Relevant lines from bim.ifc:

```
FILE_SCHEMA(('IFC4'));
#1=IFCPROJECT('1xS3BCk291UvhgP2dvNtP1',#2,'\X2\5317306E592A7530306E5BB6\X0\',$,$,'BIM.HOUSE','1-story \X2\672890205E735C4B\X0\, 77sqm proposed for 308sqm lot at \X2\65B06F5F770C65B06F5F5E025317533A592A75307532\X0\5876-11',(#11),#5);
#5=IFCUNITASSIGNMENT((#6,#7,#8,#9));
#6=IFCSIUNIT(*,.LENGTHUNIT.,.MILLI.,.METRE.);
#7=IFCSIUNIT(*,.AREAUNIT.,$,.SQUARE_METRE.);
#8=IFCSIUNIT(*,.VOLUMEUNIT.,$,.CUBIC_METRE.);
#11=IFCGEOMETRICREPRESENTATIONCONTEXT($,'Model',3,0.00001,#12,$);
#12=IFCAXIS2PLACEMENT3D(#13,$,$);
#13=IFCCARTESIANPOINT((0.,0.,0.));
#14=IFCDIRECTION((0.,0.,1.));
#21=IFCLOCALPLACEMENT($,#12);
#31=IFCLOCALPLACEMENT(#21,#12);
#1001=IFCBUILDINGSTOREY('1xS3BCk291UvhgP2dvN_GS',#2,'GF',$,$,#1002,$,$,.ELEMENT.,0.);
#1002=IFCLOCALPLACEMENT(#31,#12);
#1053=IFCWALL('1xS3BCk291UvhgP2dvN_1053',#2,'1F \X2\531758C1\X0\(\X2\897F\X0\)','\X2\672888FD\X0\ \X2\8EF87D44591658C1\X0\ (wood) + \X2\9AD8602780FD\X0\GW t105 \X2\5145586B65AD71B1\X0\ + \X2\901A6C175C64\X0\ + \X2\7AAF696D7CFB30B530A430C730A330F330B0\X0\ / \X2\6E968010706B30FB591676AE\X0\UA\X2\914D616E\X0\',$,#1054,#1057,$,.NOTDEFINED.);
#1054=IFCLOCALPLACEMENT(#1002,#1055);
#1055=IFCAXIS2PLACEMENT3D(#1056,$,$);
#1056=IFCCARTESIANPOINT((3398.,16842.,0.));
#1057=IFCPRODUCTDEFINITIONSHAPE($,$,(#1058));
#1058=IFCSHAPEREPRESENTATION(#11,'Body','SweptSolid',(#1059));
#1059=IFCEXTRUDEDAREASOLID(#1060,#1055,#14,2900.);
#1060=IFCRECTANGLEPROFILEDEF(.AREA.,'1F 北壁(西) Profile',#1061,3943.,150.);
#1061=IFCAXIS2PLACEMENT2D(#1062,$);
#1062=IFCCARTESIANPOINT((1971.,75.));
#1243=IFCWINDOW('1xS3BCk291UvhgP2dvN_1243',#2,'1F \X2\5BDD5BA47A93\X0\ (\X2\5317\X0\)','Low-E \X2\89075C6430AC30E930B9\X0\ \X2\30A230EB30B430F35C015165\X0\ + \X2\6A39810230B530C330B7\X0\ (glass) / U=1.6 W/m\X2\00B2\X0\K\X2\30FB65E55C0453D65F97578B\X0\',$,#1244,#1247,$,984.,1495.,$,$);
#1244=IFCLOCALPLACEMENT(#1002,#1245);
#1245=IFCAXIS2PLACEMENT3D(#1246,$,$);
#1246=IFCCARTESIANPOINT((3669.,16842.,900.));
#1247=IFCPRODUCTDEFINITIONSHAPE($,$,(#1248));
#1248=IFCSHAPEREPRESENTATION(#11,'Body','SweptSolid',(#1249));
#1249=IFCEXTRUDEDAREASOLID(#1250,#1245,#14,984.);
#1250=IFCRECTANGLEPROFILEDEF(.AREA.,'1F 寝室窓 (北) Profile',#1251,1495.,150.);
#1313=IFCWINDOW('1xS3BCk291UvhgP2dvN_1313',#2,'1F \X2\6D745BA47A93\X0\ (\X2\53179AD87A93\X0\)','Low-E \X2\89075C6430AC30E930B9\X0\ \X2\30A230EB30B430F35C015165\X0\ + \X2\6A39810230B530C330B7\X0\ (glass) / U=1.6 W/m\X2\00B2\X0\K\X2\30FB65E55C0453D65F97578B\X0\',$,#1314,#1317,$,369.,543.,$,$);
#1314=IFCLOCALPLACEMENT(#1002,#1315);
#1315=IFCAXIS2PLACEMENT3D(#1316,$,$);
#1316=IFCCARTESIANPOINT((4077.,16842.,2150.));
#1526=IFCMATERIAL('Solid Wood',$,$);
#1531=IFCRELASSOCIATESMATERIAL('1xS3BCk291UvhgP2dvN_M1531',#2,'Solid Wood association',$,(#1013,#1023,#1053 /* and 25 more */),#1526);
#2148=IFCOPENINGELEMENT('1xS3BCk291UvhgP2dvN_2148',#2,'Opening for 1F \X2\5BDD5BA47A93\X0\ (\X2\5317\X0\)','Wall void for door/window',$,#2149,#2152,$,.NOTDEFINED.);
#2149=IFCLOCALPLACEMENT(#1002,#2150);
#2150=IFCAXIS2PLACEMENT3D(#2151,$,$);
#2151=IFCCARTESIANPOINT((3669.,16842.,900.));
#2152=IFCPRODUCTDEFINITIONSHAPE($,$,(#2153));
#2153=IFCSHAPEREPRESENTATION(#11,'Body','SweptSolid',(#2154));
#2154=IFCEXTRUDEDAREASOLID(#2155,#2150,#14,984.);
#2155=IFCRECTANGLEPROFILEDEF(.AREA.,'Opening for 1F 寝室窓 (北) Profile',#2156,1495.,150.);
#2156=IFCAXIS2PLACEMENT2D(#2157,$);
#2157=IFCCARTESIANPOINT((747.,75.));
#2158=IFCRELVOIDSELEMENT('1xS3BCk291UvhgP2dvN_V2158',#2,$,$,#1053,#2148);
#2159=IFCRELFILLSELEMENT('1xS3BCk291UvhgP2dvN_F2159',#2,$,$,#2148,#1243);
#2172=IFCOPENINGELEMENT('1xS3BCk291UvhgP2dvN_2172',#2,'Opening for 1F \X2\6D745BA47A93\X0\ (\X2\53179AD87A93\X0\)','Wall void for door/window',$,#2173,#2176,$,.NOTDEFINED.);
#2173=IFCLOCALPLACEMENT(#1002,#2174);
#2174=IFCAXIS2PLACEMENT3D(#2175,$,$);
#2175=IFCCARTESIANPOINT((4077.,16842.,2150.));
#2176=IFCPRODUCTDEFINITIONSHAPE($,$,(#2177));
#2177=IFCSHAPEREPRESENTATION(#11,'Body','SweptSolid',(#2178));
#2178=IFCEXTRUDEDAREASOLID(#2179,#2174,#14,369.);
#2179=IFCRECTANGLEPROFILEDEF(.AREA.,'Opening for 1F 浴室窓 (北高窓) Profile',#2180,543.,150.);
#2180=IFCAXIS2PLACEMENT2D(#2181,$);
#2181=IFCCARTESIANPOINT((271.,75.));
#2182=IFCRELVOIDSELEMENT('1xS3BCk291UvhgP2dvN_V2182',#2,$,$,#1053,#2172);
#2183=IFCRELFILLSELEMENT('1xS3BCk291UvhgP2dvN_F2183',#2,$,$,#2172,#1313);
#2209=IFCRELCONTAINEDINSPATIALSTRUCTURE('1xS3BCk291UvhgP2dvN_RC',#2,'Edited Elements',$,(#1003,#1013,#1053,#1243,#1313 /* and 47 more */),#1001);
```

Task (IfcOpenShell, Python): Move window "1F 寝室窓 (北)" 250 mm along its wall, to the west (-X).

```python
import ifcopenshell
import ifcopenshell.api.geometry
import ifcopenshell.util.placement

model = ifcopenshell.open("bim.ifc")

window = model.by_guid("1xS3BCk291UvhgP2dvN_1243")
opening = window.FillsVoids[0].RelatingOpeningElement
wall = opening.VoidsElements[0].RelatingBuildingElement

wall_matrix = ifcopenshell.util.placement.get_local_placement(wall.ObjectPlacement)
shift = wall_matrix[:3, 0] * -250.0
before = ifcopenshell.util.placement.get_local_placement(window.ObjectPlacement)[:3, 3].copy()

# The window is not placed relative to its opening, so move both.
for product in (opening, window):
    matrix = ifcopenshell.util.placement.get_local_placement(product.ObjectPlacement)
    matrix[:3, 3] += shift
    ifcopenshell.api.geometry.edit_object_placement(model, product=product, matrix=matrix, is_si=False)

after = ifcopenshell.util.placement.get_local_placement(window.ObjectPlacement)[:3, 3]
print("window moved by", (after - before).round(3) + 0.0)

model.write("bim_rev.ifc")
```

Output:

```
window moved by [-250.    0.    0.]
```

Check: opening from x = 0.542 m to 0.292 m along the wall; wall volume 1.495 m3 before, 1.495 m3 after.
